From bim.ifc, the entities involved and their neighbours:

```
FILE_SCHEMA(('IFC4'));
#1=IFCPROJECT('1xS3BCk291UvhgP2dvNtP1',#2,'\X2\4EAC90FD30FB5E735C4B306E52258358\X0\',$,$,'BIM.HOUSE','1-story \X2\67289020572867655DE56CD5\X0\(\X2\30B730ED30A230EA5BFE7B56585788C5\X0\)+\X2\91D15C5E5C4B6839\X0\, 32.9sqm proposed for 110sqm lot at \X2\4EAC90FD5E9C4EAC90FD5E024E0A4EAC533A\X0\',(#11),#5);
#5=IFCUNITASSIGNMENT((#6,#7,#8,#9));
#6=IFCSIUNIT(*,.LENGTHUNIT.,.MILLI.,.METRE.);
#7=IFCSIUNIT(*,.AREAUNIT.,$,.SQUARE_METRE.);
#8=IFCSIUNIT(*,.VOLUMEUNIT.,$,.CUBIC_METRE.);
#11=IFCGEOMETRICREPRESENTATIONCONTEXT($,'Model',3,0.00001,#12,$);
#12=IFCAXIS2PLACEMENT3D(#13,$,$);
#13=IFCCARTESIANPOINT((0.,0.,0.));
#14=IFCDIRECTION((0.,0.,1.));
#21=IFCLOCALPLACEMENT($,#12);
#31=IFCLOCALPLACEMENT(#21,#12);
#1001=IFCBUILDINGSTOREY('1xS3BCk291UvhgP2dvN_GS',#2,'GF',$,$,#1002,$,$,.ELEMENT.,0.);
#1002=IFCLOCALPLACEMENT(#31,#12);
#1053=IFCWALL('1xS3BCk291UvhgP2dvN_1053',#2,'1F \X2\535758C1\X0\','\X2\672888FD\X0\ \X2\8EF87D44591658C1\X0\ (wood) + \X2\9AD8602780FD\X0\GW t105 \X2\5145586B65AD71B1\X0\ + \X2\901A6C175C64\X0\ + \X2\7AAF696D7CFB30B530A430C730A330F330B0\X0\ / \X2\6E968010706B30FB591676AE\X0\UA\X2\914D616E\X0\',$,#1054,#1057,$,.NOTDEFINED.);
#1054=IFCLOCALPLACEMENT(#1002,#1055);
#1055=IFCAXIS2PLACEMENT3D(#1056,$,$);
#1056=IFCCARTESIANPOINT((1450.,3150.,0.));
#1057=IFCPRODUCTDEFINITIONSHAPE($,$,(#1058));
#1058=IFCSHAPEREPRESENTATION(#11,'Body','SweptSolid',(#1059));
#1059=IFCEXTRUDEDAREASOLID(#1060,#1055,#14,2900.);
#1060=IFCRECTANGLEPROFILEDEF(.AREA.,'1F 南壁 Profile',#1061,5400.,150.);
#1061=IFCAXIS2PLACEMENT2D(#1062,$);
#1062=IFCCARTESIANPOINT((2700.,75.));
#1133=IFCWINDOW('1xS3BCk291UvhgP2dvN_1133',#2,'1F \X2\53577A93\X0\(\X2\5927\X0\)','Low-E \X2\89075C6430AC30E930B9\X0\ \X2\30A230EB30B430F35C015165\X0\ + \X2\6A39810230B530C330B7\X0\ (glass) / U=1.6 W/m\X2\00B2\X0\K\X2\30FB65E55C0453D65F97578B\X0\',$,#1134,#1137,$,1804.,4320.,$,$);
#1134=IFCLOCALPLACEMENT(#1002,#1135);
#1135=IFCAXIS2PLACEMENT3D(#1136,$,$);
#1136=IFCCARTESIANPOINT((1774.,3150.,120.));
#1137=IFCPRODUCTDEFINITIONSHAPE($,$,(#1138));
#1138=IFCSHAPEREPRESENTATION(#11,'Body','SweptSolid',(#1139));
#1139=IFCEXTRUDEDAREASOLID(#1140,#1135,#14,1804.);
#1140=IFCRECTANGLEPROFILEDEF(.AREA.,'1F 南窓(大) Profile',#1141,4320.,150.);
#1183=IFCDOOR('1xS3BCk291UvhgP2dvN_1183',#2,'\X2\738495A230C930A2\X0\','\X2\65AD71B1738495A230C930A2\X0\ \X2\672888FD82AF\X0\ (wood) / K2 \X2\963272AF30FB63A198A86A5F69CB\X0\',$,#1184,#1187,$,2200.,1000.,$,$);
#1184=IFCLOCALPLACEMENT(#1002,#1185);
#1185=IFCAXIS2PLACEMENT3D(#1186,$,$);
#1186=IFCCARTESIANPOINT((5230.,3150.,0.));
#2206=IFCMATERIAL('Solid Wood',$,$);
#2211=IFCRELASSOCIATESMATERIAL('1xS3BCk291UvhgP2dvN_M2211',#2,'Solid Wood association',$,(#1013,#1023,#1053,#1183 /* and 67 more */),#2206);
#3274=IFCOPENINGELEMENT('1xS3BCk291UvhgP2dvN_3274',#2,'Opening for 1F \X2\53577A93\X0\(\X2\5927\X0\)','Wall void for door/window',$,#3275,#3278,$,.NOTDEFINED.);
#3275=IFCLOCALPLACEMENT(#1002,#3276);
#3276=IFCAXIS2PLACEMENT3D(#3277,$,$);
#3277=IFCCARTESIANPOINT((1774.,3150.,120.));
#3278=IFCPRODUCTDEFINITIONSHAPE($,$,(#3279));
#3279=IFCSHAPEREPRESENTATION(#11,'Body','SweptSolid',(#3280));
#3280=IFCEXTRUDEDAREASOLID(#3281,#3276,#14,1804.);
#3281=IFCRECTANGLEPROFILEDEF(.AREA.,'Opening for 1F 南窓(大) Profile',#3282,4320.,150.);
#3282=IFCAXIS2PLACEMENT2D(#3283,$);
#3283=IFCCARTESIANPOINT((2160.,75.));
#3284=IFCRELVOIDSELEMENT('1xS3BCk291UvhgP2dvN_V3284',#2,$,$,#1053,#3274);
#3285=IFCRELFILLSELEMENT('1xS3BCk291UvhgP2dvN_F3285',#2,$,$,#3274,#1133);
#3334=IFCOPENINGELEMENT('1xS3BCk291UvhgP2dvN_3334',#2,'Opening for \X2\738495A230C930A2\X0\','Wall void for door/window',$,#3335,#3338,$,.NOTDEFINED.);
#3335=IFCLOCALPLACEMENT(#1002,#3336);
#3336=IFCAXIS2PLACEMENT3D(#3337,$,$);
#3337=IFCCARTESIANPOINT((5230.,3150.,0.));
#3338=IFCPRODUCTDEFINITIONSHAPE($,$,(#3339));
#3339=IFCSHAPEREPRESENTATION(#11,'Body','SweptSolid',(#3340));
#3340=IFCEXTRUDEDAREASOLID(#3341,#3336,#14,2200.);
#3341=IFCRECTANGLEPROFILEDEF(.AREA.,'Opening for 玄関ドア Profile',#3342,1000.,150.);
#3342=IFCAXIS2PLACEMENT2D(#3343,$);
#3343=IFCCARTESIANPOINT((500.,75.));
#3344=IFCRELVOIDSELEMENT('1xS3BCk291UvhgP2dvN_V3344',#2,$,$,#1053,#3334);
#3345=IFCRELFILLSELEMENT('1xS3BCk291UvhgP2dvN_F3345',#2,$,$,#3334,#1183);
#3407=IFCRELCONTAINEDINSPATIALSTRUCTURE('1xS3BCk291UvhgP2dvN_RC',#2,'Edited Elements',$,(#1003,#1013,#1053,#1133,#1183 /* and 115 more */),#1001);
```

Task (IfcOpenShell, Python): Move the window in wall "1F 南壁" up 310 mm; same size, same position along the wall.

```python
import numpy as np
import ifcopenshell
import ifcopenshell.api.geometry
import ifcopenshell.util.placement
import ifcopenshell.util.unit

model = ifcopenshell.open("bim.ifc")
unit_scale = ifcopenshell.util.unit.calculate_unit_scale(model)

window = model.by_guid("1xS3BCk291UvhgP2dvN_1133")
opening = window.FillsVoids[0].RelatingOpeningElement
dz = 310.0

shift = np.array([0.0, 0.0, dz])
# The window is not placed relative to its opening, so move both.
for product in (opening, window):
    matrix = ifcopenshell.util.placement.get_local_placement(product.ObjectPlacement)
    matrix[:3, 3] += shift
    ifcopenshell.api.geometry.edit_object_placement(model, product=product, matrix=matrix, is_si=False)

print(f"moved by {dz * unit_scale:+.3f} m")

model.write("bim_v2.ifc")
```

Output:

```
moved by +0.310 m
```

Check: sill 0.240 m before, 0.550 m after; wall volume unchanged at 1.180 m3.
